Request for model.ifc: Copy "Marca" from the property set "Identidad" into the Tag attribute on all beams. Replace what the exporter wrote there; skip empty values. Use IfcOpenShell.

First a look at what the model holds.

```python
import ifcopenshell
import ifcopenshell.util.element

model = ifcopenshell.open("model.ifc")
print(model.schema)
beams = model.by_type("IfcBeam")
print(len(beams), "beams")
for e in beams[:8]:
    source = ifcopenshell.util.element.get_pset(e, "Identidad", "Marca")
    target = e.Tag
    print(e.id(), repr(source), repr(target), sep=" | ")
```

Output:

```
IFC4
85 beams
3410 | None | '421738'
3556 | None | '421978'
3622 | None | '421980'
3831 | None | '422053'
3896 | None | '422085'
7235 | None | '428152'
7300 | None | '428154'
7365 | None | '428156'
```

```python
import ifcopenshell
import ifcopenshell.util.element

model = ifcopenshell.open("model.ifc")

count = 0
for e in model.by_type("IfcBeam"):
    value = ifcopenshell.util.element.get_pset(e, "Identidad", "Marca")
    current = e.Tag
    if not value or not value.strip() or current == value:
        continue
    e.Tag = value
    count += 1

print(count, "beams updated")

model.write("model-out.ifc")
```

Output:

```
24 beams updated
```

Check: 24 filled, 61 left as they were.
